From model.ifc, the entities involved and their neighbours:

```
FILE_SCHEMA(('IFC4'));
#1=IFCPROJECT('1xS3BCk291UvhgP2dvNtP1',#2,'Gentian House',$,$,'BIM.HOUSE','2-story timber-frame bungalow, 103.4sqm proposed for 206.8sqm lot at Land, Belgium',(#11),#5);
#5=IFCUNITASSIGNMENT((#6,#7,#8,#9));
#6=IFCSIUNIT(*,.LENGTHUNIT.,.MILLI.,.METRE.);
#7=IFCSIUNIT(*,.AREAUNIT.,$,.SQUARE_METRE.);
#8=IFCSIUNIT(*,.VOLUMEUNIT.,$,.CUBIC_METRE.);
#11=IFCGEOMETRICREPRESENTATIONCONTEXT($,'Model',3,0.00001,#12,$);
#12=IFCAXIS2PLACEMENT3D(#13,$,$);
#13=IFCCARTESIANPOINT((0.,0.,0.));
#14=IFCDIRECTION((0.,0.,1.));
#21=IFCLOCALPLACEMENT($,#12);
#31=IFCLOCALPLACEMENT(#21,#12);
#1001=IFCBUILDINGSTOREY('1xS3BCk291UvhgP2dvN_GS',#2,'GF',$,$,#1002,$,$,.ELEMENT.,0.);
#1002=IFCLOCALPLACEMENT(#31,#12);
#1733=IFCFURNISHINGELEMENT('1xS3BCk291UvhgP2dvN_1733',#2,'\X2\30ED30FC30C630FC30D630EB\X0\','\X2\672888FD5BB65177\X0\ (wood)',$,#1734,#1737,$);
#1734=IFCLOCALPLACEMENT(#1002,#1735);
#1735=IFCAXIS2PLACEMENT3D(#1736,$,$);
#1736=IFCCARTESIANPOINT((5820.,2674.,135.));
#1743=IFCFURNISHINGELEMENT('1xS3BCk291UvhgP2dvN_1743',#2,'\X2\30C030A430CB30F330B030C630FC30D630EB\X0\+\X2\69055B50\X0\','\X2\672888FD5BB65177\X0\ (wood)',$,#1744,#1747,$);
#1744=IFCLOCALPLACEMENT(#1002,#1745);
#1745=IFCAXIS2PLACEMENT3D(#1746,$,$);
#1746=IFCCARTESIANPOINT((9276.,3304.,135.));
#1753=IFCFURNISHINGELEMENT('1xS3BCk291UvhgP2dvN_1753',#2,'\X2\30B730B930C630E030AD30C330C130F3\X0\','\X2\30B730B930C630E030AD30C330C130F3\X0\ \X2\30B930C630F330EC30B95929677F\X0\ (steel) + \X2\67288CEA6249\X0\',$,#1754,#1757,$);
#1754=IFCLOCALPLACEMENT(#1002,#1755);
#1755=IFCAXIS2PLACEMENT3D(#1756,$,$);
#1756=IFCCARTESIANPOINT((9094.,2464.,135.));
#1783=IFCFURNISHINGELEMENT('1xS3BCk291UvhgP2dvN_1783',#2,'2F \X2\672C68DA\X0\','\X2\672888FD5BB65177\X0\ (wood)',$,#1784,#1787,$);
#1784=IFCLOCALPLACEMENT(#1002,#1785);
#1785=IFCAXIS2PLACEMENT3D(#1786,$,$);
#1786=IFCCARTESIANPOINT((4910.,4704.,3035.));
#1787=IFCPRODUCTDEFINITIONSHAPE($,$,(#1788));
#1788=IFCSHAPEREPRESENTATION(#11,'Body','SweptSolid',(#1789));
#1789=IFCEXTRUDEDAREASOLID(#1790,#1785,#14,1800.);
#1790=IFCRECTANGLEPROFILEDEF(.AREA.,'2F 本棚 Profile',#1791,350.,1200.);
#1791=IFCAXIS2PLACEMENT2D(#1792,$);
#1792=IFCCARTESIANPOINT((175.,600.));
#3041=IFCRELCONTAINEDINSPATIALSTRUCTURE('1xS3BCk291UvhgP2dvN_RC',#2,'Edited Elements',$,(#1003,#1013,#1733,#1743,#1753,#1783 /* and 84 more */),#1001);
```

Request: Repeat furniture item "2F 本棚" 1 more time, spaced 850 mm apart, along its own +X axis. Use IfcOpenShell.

```python
import ifcopenshell
import ifcopenshell.api.geometry
import ifcopenshell.api.root
import ifcopenshell.util.element
import ifcopenshell.util.placement
import ifcopenshell.util.unit

model = ifcopenshell.open("model.ifc")
unit_scale = ifcopenshell.util.unit.calculate_unit_scale(model)


def reuse_history(source, copy):
    """copy_class also copies each property set's owner history, people and application; keep the originals."""
    for rel in copy.IsDefinedBy:
        if rel.is_a("IfcRelDefinesByProperties") and (history := rel.RelatingPropertyDefinition.OwnerHistory):
            rel.RelatingPropertyDefinition.OwnerHistory = source.OwnerHistory
            ifcopenshell.util.element.remove_deep2(model, history)


source = model.by_guid("1xS3BCk291UvhgP2dvN_1783")
base = ifcopenshell.util.placement.get_local_placement(source.ObjectPlacement)
step = base[:3, 0] * 0.85 / unit_scale

for i in range(1, 2):
    copy = ifcopenshell.api.root.copy_class(model, product=source)
    copy.Representation = ifcopenshell.util.element.copy_deep(
        model, source.Representation, exclude=["IfcGeometricRepresentationContext", "IfcRepresentationMap"]
    )
    reuse_history(source, copy)
    matrix = base.copy()
    matrix[:3, 3] += i * step
    print("added at", matrix[:3, 3].round(3) + 0.0)
    ifcopenshell.api.geometry.edit_object_placement(model, product=copy, matrix=matrix, is_si=False)

model.write("model_updated.ifc")
```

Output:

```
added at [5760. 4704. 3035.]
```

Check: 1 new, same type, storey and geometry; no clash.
